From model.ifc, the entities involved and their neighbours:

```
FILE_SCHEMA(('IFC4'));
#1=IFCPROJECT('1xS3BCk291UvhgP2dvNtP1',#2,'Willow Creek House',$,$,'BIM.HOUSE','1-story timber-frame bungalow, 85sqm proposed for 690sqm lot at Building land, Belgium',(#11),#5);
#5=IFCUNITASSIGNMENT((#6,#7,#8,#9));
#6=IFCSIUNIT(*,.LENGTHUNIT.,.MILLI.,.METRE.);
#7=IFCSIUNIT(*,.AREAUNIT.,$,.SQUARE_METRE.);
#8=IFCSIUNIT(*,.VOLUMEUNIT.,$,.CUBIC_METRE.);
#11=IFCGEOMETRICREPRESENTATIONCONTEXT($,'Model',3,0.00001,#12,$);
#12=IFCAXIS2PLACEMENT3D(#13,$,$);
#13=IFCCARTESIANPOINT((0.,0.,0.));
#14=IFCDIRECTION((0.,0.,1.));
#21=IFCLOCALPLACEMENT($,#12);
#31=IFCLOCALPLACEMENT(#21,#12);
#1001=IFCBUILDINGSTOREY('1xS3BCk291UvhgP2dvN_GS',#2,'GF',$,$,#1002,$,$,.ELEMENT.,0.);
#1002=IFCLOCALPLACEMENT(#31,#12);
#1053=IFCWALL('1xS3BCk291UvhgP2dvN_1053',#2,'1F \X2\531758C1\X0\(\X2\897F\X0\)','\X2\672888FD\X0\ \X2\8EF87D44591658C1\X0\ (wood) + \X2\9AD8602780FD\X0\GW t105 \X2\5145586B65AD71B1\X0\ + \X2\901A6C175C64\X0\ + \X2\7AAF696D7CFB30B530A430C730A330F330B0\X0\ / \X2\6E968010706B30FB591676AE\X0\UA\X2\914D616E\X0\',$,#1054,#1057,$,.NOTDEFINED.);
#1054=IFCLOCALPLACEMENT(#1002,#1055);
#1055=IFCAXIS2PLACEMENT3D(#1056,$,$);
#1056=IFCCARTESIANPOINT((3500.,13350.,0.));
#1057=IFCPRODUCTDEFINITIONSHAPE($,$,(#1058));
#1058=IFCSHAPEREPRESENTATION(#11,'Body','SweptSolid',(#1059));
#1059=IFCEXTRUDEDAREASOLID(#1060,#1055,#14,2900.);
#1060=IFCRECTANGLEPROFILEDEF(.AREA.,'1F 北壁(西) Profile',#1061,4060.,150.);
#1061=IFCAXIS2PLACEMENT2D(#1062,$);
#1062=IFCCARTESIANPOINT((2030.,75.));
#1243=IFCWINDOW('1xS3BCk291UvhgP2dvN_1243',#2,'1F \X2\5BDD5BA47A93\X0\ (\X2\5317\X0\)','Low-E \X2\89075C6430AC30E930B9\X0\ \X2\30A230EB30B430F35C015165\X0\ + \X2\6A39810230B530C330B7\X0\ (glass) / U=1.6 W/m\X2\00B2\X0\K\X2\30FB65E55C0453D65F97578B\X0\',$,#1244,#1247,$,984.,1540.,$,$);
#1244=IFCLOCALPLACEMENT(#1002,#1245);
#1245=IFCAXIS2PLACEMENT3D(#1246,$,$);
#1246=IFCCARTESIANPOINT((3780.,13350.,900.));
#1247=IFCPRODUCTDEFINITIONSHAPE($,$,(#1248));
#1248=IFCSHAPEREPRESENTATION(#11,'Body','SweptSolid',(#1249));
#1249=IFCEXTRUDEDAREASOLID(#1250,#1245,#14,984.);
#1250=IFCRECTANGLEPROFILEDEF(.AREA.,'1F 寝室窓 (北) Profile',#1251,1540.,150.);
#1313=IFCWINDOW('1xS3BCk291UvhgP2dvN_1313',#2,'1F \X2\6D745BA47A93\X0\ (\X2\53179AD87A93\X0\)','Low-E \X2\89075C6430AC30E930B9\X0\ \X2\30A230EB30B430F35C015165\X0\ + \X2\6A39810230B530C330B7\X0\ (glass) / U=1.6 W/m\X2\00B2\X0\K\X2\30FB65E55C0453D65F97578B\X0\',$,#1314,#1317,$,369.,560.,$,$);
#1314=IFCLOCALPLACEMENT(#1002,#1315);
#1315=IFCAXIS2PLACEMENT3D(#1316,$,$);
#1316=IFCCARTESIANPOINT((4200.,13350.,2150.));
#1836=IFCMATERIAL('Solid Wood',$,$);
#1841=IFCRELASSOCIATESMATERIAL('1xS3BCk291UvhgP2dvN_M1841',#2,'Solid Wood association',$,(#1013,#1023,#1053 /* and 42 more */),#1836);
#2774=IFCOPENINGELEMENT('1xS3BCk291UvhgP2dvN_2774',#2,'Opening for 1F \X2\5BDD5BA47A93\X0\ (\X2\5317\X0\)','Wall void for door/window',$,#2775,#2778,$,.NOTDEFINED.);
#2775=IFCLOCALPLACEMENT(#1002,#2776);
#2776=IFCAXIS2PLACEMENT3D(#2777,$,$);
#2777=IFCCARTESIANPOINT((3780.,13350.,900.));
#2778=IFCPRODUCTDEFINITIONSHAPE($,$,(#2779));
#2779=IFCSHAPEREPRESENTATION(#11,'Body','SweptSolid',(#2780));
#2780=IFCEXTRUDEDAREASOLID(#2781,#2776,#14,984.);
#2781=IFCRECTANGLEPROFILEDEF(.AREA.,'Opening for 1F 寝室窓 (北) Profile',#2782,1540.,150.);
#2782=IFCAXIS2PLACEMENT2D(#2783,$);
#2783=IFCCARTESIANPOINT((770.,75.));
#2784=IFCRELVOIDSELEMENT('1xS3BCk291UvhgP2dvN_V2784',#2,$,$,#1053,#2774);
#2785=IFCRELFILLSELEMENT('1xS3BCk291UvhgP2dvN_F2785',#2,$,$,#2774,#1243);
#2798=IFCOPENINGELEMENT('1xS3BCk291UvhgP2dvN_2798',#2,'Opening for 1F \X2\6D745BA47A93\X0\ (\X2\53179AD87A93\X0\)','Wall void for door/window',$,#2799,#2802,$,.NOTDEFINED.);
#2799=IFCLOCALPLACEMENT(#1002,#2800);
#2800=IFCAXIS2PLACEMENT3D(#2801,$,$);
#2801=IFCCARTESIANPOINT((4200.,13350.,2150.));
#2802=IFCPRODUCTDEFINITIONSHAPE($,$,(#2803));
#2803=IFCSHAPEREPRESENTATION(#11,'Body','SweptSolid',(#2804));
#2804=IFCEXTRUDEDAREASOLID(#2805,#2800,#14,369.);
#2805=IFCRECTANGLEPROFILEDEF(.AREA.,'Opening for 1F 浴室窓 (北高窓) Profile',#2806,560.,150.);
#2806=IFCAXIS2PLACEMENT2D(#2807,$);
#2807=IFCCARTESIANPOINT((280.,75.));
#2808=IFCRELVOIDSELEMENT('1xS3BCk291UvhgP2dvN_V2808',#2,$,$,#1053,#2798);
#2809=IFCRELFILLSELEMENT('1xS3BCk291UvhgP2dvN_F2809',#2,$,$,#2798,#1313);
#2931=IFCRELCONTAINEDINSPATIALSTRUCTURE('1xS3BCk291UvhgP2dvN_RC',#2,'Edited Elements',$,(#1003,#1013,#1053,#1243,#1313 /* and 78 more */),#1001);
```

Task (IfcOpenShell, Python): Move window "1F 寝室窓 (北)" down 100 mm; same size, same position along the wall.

```python
import numpy as np
import ifcopenshell
import ifcopenshell.api.geometry
import ifcopenshell.util.placement
import ifcopenshell.util.unit

model = ifcopenshell.open("model.ifc")
unit_scale = ifcopenshell.util.unit.calculate_unit_scale(model)

window = model.by_id(1243)
opening = window.FillsVoids[0].RelatingOpeningElement
dz = -0.1 / unit_scale

shift = np.array([0.0, 0.0, dz])
# The window is not placed relative to its opening, so move both.
for product in (opening, window):
    matrix = ifcopenshell.util.placement.get_local_placement(product.ObjectPlacement)
    matrix[:3, 3] += shift
    ifcopenshell.api.geometry.edit_object_placement(model, product=product, matrix=matrix, is_si=False)

print(f"moved by {dz * unit_scale:+.3f} m")

model.write("model-out.ifc")
```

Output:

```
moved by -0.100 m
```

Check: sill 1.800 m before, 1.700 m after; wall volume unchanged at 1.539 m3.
